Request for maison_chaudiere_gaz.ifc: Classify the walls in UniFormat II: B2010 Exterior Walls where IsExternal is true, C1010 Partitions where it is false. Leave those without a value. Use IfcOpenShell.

First a look at what the model holds.

```python
import ifcopenshell
import ifcopenshell.util.element

model = ifcopenshell.open("maison_chaudiere_gaz.ifc")
print(model.schema)
print("classifications:", [c.Name for c in model.by_type("IfcClassification")])
values = [ifcopenshell.util.element.get_pset(e, "Pset_WallCommon", "IsExternal") for e in model.by_type("IfcWall")]
for value in (True, False, None):
    print("IsExternal", value, values.count(value))
```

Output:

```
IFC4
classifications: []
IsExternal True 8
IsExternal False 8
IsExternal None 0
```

```python
import ifcopenshell
import ifcopenshell.api.classification
import ifcopenshell.util.element

model = ifcopenshell.open("maison_chaudiere_gaz.ifc")

system = ifcopenshell.api.classification.add_classification(model, classification="UniFormat II")

walls = model.by_type("IfcWall")
external = {e: ifcopenshell.util.element.get_pset(e, "Pset_WallCommon", "IsExternal") for e in walls}
for flag, code, name in ((True, "B2010", "Exterior Walls"), (False, "C1010", "Partitions")):
    products = [e for e in walls if external[e] is flag]
    ifcopenshell.api.classification.add_reference(
        model, products=products, classification=system, identification=code, name=name
    )
    print(code, len(products))

model.write("maison_chaudiere_gaz_v2.ifc")
```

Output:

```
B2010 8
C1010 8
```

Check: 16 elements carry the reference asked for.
